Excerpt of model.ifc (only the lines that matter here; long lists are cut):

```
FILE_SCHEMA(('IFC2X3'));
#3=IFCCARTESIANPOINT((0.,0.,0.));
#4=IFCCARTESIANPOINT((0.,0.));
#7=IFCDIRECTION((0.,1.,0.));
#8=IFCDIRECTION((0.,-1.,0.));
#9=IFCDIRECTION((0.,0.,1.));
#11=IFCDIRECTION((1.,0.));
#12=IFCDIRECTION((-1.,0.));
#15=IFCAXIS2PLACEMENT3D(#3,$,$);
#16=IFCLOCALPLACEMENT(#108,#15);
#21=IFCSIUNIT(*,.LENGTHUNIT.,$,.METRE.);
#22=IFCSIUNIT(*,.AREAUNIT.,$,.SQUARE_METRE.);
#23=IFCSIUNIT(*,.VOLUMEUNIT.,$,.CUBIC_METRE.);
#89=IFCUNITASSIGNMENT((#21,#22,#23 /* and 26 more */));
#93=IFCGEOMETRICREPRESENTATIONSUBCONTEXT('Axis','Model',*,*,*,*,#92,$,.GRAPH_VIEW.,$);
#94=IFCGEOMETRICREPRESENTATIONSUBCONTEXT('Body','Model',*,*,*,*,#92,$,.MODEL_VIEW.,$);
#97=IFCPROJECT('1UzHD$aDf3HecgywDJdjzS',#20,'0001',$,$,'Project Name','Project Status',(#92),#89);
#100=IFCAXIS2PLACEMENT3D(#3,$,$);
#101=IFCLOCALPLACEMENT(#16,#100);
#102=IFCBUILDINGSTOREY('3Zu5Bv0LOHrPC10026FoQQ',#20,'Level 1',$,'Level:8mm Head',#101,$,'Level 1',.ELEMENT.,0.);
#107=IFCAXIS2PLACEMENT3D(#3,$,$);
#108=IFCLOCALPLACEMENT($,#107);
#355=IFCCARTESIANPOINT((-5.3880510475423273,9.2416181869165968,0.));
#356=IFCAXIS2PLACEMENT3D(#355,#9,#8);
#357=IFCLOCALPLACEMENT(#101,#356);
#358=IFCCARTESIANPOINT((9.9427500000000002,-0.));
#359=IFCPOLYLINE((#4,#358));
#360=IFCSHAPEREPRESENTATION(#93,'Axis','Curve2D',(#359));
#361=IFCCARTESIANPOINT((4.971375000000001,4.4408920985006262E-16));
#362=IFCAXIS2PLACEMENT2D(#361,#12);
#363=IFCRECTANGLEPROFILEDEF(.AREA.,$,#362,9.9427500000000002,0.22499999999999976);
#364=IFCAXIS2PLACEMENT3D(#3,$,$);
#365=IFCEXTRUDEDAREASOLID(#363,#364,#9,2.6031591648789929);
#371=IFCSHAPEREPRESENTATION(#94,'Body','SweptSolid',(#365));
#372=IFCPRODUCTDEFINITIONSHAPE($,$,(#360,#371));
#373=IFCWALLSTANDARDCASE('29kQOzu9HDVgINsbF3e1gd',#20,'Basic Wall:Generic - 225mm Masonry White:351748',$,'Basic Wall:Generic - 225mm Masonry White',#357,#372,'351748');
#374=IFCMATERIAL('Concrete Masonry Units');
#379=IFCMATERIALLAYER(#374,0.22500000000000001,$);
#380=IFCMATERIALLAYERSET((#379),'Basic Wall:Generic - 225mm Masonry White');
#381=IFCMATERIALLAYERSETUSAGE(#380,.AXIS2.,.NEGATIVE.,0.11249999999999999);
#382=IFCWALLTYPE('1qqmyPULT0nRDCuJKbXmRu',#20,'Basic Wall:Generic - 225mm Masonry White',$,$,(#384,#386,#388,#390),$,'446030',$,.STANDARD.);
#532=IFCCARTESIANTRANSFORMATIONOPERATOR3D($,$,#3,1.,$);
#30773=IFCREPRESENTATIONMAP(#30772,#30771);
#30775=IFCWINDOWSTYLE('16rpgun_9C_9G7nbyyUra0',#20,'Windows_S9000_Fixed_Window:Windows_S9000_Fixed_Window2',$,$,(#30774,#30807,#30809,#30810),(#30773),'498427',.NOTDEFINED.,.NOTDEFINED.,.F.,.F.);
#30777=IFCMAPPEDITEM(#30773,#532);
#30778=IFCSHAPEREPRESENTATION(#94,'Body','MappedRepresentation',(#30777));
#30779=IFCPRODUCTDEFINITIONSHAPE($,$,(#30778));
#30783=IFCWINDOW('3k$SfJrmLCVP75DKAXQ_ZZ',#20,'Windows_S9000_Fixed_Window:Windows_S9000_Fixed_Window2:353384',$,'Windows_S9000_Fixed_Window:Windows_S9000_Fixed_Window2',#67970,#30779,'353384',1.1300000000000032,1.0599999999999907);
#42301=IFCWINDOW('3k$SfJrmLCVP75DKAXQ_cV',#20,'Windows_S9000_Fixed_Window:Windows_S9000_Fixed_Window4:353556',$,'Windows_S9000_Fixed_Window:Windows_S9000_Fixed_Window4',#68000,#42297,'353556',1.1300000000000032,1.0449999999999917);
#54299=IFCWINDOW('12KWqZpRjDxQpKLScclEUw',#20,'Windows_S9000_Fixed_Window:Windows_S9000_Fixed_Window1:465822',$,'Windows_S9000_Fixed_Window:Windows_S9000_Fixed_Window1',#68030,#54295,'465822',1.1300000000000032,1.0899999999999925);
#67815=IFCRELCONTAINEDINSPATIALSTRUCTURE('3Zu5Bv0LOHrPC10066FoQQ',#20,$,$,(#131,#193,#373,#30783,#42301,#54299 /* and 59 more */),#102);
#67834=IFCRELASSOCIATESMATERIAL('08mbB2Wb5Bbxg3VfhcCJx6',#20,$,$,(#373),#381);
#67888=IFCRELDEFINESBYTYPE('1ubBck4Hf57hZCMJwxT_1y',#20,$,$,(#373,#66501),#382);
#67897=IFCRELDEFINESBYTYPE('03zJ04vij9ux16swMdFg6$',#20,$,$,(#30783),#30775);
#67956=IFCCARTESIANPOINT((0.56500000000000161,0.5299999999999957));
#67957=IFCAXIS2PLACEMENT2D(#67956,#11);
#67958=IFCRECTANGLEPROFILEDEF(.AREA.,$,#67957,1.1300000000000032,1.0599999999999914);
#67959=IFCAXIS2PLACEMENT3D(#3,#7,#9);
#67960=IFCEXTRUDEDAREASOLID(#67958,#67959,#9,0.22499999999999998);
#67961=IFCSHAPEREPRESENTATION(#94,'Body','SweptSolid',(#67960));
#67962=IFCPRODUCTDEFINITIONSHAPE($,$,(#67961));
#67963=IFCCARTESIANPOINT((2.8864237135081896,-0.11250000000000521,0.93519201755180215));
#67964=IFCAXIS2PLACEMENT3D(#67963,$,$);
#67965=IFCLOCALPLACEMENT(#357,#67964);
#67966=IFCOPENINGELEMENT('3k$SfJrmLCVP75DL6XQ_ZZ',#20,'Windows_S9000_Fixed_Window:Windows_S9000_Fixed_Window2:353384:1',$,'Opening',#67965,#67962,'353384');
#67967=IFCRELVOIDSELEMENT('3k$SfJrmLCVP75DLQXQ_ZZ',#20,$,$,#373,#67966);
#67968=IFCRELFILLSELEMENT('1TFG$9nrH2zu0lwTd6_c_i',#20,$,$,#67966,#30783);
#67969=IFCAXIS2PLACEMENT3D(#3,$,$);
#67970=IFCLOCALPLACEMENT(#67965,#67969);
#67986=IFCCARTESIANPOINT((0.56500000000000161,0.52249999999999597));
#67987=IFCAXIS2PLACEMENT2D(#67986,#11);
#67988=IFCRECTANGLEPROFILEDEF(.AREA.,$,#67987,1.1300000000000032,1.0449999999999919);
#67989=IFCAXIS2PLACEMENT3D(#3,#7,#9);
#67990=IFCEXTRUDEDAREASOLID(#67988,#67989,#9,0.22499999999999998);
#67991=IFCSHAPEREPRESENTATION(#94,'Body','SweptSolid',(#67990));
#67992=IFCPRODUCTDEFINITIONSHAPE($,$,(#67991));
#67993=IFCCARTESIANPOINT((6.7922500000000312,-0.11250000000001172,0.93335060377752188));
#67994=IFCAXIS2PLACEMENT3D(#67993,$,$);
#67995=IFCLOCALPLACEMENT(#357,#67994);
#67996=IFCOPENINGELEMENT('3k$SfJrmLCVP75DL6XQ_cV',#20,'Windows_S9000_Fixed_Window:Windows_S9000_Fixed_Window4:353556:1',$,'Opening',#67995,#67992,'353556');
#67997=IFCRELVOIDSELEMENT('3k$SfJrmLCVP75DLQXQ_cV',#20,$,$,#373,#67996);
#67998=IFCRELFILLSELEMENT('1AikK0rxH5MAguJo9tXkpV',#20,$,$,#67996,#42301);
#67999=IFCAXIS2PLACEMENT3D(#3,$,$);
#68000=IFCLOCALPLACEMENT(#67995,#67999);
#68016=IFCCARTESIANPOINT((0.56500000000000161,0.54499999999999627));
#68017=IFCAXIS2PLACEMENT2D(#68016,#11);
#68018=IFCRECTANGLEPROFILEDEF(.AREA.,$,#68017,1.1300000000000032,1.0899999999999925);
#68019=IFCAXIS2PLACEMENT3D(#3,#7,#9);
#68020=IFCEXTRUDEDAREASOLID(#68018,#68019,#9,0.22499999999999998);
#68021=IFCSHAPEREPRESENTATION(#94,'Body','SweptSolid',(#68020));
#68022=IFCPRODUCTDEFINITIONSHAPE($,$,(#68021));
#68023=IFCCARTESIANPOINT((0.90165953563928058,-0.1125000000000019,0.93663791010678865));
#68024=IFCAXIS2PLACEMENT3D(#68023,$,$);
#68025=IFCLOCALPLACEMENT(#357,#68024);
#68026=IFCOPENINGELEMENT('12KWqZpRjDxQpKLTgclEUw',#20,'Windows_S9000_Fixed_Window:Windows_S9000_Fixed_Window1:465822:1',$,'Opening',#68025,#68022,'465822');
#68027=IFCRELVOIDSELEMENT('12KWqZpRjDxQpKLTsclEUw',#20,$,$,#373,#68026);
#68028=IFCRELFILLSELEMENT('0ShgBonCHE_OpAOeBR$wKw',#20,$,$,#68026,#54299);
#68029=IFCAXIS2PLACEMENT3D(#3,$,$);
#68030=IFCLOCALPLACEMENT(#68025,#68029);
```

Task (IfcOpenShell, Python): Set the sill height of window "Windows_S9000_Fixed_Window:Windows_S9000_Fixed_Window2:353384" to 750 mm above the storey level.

```python
import numpy as np
import ifcopenshell
import ifcopenshell.api.geometry
import ifcopenshell.geom
import ifcopenshell.util.element
import ifcopenshell.util.placement
import ifcopenshell.util.shape
import ifcopenshell.util.unit

model = ifcopenshell.open("model.ifc")
unit_scale = ifcopenshell.util.unit.calculate_unit_scale(model)

window = model.by_guid("3k$SfJrmLCVP75DKAXQ_ZZ")
opening = window.FillsVoids[0].RelatingOpeningElement
storey = ifcopenshell.util.element.get_container(window, ifc_class="IfcBuildingStorey")
level = ifcopenshell.util.placement.get_local_placement(storey.ObjectPlacement)[2, 3]

# The opening's origin need not be at the sill, so measure its lowest point.
shape = ifcopenshell.geom.create_shape(ifcopenshell.geom.settings(), opening)
bottom = ifcopenshell.util.shape.get_shape_bottom_elevation(shape, shape.geometry) / unit_scale
dz = level + 0.75 - bottom

shift = np.array([0.0, 0.0, dz])
# The window is placed relative to its opening, so it follows when the opening moves.
matrix = ifcopenshell.util.placement.get_local_placement(opening.ObjectPlacement)
matrix[:3, 3] += shift
ifcopenshell.api.geometry.edit_object_placement(
    model, product=opening, matrix=matrix, is_si=False, should_transform_children=True
)

print(f"moved by {dz * unit_scale:+.3f} m")

model.write("model_edited.ifc")
```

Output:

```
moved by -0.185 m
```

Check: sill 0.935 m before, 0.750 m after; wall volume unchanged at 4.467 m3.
